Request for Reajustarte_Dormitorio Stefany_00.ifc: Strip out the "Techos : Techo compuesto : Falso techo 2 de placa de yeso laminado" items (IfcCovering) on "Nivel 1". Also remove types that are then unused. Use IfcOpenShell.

First a look at what the model holds.

```python
import ifcopenshell
import ifcopenshell.util.element

model = ifcopenshell.open("Reajustarte_Dormitorio Stefany_00.ifc")
print(model.schema)
storey = next(s for s in model.by_type("IfcBuildingStorey") if s.Name == "Nivel 1")
coverings = [e for e in ifcopenshell.util.element.get_decomposition(storey) if e.is_a("IfcCovering")]
seen = {}
for e in coverings:
    element_type = ifcopenshell.util.element.get_type(e)
    name = element_type.Name if element_type not in (None, e) else None
    seen[name] = seen.get(name, 0) + 1
for name, count in sorted(seen.items(), key=str):
    print(count, "x", name)
```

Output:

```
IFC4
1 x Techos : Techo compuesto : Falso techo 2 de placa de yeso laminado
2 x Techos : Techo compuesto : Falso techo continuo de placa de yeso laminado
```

```python
import ifcopenshell
import ifcopenshell.api.root
import ifcopenshell.util.element

model = ifcopenshell.open("Reajustarte_Dormitorio Stefany_00.ifc")

storey = next(s for s in model.by_type("IfcBuildingStorey") if s.Name == "Nivel 1")
coverings = [e for e in ifcopenshell.util.element.get_decomposition(storey) if e.is_a("IfcCovering")]
targets = [e for e in coverings if (t := ifcopenshell.util.element.get_type(e)) not in (None, e) and t.Name == "Techos : Techo compuesto : Falso techo 2 de placa de yeso laminado"]
types = {ifcopenshell.util.element.get_type(e) for e in targets} - {None, *targets}

for e in targets:
    ifcopenshell.api.root.remove_product(model, product=e)
print(len(targets), "removed")

unused = [t for t in types if not ifcopenshell.util.element.get_types(t)]
for t in unused:
    ifcopenshell.api.root.remove_product(model, product=t)
print(len(unused), "unused types removed")

model.write("Reajustarte_Dormitorio Stefany_00_rev.ifc")
```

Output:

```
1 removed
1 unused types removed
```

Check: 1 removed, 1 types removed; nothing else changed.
